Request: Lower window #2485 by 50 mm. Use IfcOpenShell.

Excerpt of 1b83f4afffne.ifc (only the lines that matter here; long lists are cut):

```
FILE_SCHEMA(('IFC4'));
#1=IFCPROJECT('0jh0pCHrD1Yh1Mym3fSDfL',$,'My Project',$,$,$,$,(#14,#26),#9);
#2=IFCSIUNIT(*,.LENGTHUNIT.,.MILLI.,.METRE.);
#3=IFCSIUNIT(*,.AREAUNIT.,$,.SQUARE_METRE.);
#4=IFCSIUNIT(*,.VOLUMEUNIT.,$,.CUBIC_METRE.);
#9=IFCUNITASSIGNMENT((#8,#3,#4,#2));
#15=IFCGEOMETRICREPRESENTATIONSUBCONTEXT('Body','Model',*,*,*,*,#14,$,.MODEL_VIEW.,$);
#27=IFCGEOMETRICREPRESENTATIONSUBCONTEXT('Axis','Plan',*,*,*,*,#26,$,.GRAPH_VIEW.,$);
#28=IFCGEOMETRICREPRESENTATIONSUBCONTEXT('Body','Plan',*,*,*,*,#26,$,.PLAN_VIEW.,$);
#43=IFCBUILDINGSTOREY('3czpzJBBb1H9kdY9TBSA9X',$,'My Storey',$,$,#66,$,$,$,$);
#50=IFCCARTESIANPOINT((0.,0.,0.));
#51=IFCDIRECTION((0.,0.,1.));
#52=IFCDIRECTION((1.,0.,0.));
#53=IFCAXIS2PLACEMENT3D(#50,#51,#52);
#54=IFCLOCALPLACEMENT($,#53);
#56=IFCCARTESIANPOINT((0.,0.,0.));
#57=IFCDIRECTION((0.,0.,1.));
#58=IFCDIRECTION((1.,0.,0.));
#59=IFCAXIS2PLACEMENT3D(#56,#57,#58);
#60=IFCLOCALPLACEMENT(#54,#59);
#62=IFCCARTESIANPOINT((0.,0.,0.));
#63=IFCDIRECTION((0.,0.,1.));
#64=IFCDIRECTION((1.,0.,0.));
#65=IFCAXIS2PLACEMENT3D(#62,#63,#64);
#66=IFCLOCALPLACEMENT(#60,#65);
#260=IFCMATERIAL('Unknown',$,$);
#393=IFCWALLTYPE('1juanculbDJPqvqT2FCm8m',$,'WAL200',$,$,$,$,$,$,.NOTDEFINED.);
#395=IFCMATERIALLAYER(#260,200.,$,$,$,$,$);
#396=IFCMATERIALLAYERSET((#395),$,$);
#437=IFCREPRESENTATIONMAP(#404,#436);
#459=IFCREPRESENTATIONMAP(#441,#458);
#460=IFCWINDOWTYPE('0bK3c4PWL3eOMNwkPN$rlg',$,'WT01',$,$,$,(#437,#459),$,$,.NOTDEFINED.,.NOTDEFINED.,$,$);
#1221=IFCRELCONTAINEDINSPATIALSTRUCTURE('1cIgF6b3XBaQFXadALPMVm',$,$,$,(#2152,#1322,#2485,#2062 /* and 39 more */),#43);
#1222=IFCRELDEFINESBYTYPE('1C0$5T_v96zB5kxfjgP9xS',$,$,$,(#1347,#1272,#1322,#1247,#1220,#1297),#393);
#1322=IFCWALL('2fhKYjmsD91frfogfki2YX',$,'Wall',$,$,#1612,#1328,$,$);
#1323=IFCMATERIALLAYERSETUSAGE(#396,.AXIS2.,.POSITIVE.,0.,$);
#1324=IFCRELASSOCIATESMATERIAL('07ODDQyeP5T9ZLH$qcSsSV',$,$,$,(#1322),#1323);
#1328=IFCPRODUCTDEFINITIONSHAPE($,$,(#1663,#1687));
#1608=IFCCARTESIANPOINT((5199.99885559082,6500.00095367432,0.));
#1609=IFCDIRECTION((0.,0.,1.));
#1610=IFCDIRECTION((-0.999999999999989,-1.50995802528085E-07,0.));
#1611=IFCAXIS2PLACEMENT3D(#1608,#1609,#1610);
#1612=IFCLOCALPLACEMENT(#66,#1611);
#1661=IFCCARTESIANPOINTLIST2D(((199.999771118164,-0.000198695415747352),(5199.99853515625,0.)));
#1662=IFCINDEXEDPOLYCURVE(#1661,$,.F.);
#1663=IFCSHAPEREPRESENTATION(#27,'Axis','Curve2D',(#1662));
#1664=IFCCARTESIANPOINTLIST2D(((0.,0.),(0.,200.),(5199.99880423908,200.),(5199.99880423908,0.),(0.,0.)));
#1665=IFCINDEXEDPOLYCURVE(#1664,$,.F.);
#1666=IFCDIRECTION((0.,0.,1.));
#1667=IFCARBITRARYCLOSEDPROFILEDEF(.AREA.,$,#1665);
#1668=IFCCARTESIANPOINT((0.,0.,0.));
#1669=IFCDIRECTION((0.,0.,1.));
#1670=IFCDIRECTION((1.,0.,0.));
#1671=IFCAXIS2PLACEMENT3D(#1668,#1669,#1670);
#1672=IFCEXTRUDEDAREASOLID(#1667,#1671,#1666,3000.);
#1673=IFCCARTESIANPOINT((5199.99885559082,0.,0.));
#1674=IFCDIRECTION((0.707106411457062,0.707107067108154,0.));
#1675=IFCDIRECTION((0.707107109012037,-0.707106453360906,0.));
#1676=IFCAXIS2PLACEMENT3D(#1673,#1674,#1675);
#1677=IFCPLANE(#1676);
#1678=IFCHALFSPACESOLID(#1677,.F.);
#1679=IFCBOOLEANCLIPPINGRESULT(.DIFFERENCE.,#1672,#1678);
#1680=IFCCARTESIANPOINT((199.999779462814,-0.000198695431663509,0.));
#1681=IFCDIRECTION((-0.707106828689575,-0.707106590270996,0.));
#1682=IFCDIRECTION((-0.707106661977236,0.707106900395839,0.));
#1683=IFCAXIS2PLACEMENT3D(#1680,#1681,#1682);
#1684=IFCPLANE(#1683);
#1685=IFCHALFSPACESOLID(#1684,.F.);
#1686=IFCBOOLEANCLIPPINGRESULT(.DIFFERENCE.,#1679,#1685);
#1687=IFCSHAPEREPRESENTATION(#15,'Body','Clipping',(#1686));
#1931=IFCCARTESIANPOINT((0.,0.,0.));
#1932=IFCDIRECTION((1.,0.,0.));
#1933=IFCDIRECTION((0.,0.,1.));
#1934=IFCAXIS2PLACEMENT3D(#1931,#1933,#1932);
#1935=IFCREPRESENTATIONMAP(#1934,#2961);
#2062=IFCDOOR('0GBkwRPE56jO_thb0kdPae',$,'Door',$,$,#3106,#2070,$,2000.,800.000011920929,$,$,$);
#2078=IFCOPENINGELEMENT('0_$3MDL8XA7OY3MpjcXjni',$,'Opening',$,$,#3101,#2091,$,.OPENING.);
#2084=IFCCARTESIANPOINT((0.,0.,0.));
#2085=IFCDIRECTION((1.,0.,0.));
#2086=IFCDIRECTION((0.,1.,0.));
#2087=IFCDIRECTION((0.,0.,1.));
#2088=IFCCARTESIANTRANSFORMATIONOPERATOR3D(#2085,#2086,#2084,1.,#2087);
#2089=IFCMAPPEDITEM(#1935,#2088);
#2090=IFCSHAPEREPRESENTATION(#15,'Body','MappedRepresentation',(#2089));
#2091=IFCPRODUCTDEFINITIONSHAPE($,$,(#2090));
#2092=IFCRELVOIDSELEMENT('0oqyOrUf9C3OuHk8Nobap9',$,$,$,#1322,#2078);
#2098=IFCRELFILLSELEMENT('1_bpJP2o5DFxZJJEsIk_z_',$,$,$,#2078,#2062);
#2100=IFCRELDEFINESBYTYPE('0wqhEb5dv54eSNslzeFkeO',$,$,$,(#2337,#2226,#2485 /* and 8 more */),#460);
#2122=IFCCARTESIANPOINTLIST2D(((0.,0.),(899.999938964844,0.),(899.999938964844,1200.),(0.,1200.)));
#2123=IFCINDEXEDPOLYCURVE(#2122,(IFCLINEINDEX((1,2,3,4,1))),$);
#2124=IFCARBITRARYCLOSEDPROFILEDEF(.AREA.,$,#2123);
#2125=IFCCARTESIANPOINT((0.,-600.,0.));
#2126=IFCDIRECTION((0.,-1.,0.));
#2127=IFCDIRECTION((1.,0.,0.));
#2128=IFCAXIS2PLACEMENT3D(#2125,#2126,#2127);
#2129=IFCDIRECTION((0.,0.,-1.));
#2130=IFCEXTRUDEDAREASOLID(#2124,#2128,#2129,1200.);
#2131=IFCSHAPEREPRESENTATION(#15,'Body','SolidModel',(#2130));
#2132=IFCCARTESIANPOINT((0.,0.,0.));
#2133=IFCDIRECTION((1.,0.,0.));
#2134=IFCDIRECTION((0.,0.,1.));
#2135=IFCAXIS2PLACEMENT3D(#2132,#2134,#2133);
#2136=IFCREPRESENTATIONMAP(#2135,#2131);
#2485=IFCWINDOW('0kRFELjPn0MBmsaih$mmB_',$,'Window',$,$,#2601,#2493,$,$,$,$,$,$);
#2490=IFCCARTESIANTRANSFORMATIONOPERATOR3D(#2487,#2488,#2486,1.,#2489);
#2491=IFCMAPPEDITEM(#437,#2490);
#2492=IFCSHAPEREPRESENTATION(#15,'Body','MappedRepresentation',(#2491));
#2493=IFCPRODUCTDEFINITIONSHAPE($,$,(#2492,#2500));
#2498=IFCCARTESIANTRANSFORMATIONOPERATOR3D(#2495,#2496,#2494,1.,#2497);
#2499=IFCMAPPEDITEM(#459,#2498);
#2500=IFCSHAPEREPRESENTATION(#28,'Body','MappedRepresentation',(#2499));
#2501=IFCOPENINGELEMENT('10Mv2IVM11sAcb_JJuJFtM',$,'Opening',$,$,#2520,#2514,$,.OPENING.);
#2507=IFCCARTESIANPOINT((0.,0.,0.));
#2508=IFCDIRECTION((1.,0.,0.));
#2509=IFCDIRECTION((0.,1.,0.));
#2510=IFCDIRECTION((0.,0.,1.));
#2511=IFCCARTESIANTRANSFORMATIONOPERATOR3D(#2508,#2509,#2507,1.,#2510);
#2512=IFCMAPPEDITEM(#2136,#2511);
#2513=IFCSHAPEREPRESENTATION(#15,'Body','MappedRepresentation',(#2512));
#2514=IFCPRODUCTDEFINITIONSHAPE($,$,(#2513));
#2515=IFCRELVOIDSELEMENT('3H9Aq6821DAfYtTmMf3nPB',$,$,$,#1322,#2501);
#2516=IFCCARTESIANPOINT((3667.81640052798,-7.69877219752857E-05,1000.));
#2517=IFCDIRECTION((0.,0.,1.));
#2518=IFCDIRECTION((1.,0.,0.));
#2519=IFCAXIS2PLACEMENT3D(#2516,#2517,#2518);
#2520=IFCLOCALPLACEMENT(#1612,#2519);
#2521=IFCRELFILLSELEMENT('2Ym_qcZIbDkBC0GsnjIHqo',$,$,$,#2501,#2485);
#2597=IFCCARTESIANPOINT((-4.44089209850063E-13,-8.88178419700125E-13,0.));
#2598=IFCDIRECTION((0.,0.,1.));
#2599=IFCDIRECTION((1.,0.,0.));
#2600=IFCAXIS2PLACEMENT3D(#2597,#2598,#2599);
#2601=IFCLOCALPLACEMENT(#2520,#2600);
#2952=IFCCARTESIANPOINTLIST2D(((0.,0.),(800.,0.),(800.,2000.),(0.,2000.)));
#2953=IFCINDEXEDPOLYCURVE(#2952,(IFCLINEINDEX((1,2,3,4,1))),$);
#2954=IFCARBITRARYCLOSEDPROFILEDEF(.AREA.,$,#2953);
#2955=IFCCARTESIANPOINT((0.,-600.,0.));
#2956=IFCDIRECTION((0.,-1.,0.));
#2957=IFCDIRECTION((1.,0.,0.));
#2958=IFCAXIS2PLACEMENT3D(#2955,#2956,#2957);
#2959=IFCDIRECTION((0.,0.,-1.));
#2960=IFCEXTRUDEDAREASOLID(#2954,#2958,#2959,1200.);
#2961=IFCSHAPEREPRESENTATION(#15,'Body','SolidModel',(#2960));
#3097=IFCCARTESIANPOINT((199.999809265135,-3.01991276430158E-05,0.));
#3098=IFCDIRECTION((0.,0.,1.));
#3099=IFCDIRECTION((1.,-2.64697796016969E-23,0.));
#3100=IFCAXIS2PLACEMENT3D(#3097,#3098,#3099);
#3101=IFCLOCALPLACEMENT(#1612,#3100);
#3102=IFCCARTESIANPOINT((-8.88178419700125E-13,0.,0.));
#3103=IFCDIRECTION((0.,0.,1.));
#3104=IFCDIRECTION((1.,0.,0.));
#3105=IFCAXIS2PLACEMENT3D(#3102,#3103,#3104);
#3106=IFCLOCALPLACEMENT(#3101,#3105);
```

```python
import numpy as np
import ifcopenshell
import ifcopenshell.api.geometry
import ifcopenshell.util.placement
import ifcopenshell.util.unit

model = ifcopenshell.open("1b83f4afffne.ifc")
unit_scale = ifcopenshell.util.unit.calculate_unit_scale(model)

window = model.by_guid("0kRFELjPn0MBmsaih$mmB_")
opening = window.FillsVoids[0].RelatingOpeningElement
dz = -0.05 / unit_scale

shift = np.array([0.0, 0.0, dz])
# The window is placed relative to its opening, so it follows when the opening moves.
matrix = ifcopenshell.util.placement.get_local_placement(opening.ObjectPlacement)
matrix[:3, 3] += shift
ifcopenshell.api.geometry.edit_object_placement(
    model, product=opening, matrix=matrix, is_si=False, should_transform_children=True
)

print(f"moved by {dz * unit_scale:+.3f} m")

model.write("1b83f4afffne_v2.ifc")
```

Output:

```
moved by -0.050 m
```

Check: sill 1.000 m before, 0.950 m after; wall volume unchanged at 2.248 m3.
